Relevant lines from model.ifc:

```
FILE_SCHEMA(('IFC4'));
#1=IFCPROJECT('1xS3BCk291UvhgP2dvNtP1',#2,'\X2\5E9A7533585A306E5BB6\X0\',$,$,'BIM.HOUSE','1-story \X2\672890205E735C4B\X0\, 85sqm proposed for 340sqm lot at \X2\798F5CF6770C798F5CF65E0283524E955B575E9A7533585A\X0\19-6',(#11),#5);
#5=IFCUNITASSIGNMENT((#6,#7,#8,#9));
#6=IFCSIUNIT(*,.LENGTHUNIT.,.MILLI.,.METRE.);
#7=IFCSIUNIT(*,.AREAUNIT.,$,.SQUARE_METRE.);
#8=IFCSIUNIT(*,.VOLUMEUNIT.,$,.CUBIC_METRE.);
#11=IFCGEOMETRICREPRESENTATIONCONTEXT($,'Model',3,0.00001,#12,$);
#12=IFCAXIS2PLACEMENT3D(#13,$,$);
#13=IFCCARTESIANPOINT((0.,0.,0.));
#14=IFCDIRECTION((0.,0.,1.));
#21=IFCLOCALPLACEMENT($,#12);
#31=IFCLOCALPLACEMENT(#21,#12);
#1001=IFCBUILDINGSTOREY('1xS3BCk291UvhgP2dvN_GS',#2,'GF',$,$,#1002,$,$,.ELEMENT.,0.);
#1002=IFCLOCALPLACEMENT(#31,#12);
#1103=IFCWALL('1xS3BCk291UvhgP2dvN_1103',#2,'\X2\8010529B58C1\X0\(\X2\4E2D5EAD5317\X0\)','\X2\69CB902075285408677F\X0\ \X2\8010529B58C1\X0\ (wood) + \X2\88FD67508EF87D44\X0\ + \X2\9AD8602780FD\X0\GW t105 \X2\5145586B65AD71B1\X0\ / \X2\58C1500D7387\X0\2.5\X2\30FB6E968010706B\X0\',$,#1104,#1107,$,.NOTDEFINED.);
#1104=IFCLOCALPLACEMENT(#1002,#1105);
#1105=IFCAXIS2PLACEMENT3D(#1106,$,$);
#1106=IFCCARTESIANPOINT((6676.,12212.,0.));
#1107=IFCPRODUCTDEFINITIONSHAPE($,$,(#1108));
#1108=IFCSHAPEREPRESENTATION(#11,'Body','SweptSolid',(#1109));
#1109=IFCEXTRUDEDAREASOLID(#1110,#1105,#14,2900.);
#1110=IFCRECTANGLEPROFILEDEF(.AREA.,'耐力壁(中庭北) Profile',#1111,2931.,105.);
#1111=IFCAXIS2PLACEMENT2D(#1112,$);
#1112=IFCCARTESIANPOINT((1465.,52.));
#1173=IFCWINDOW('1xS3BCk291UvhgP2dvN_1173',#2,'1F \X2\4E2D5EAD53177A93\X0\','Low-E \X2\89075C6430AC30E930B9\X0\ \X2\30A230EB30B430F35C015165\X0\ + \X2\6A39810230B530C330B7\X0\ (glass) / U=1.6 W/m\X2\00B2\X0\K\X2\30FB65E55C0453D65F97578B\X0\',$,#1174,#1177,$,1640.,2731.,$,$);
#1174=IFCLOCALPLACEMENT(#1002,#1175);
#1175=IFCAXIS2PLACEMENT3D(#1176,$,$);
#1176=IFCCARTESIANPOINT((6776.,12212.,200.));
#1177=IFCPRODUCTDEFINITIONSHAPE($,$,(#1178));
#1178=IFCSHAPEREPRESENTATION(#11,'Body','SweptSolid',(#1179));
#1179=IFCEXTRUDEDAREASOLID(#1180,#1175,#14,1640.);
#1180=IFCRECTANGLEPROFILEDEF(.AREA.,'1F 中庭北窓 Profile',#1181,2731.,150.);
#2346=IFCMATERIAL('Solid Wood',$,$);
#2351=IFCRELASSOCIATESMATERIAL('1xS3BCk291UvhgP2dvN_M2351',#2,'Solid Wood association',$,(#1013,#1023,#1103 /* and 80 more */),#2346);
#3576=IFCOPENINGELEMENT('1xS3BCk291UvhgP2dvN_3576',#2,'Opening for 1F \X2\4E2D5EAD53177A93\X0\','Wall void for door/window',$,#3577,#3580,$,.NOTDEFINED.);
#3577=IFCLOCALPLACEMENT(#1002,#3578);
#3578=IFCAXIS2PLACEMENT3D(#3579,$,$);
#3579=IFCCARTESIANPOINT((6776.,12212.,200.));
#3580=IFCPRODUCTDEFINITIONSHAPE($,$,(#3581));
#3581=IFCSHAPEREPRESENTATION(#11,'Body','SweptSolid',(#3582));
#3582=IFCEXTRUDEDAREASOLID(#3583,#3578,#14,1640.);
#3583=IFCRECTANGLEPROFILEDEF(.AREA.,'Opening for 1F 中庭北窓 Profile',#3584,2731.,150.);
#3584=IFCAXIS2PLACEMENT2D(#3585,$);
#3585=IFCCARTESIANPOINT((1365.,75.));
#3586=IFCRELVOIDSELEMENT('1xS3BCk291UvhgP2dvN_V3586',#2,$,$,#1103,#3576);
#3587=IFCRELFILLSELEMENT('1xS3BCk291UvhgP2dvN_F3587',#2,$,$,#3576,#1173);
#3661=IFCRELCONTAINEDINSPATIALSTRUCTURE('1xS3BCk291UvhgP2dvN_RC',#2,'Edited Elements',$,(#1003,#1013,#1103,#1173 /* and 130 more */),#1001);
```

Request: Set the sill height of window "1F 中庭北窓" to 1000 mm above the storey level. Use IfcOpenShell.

```python
import numpy as np
import ifcopenshell
import ifcopenshell.api.geometry
import ifcopenshell.geom
import ifcopenshell.util.element
import ifcopenshell.util.placement
import ifcopenshell.util.shape
import ifcopenshell.util.unit

model = ifcopenshell.open("model.ifc")
unit_scale = ifcopenshell.util.unit.calculate_unit_scale(model)

window = model.by_guid("1xS3BCk291UvhgP2dvN_1173")
opening = window.FillsVoids[0].RelatingOpeningElement
storey = ifcopenshell.util.element.get_container(window, ifc_class="IfcBuildingStorey")
level = ifcopenshell.util.placement.get_local_placement(storey.ObjectPlacement)[2, 3]

# The opening's origin need not be at the sill, so measure its lowest point.
shape = ifcopenshell.geom.create_shape(ifcopenshell.geom.settings(), opening)
bottom = ifcopenshell.util.shape.get_shape_bottom_elevation(shape, shape.geometry) / unit_scale
dz = level + 1 / unit_scale - bottom

shift = np.array([0.0, 0.0, dz])
# The window is not placed relative to its opening, so move both.
for product in (opening, window):
    matrix = ifcopenshell.util.placement.get_local_placement(product.ObjectPlacement)
    matrix[:3, 3] += shift
    ifcopenshell.api.geometry.edit_object_placement(model, product=product, matrix=matrix, is_si=False)

print(f"moved by {dz * unit_scale:+.3f} m")

model.write("model-out.ifc")
```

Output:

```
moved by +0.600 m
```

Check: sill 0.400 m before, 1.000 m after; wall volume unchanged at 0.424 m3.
